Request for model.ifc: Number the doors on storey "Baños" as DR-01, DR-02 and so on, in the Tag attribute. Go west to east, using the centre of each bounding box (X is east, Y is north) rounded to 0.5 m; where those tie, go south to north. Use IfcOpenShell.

First a look at what the model holds.

```python
import ifcopenshell
import ifcopenshell.util.element
import ifcopenshell.util.placement

model = ifcopenshell.open("model.ifc")
print(model.schema)
storey = next(s for s in model.by_type("IfcBuildingStorey") if s.Name == "Baños")
doors = [e for e in ifcopenshell.util.element.get_decomposition(storey) if e.is_a("IfcDoor")]
for e in sorted(doors, key=lambda e: e.id()):
    origin = ifcopenshell.util.placement.get_local_placement(e.ObjectPlacement)[:3, 3]
    print(e.id(), e.Tag, e.Name, origin.round(2) + 0.0, sep=" | ")
```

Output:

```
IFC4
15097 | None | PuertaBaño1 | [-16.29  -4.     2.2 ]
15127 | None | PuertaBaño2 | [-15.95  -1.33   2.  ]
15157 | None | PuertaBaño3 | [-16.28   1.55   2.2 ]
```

```python
import ifcopenshell
import ifcopenshell.geom
import ifcopenshell.util.element
import ifcopenshell.util.shape

model = ifcopenshell.open("model.ifc")
settings = ifcopenshell.geom.settings()
settings.set("use-world-coords", True)


def centre(element):
    shape = ifcopenshell.geom.create_shape(settings, element)
    return ifcopenshell.util.shape.get_bbox_centroid(shape.geometry)


storey = next(s for s in model.by_type("IfcBuildingStorey") if s.Name == "Baños")
doors = [e for e in ifcopenshell.util.element.get_decomposition(storey) if e.is_a("IfcDoor")]

# Insertion points can sit at a corner or the storey origin, so sort by the geometry (in metres).
centres = {e: centre(e) for e in doors}
doors.sort(key=lambda e: (round(centres[e][0] / 0.5), centres[e][1]))

for i, e in enumerate(doors, start=1):
    number = f"DR-{i:02d}"
    e.Tag = number
    print(e.id(), number)

model.write("model_updated.ifc")
```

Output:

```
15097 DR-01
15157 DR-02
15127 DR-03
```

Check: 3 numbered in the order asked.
